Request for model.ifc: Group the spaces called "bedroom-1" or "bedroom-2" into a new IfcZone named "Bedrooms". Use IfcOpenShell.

First a look at what the model holds.

```python
import ifcopenshell

model = ifcopenshell.open("model.ifc")
print(model.schema)
seen = {}
for space in model.by_type("IfcSpace"):
    seen[space.Name] = seen.get(space.Name, 0) + 1
for name, count in sorted(seen.items(), key=str):
    print(count, "x", name)
print("zones:", [z.Name for z in model.by_type("IfcZone")][:20])
```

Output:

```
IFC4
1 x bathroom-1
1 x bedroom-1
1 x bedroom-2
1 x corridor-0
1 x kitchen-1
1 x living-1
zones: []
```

```python
import ifcopenshell
import ifcopenshell.api.group
import ifcopenshell.api.root

model = ifcopenshell.open("model.ifc")

names = {"bedroom-1", "bedroom-2"}
spaces = [s for s in model.by_type("IfcSpace") if s.Name in names]

zone = ifcopenshell.api.root.create_entity(model, ifc_class="IfcZone", name="Bedrooms")
ifcopenshell.api.group.assign_group(model, products=spaces, group=zone)
print(len(spaces), "spaces in", zone.Name)

model.write("model_updated.ifc")
```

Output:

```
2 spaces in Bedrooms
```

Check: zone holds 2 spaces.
